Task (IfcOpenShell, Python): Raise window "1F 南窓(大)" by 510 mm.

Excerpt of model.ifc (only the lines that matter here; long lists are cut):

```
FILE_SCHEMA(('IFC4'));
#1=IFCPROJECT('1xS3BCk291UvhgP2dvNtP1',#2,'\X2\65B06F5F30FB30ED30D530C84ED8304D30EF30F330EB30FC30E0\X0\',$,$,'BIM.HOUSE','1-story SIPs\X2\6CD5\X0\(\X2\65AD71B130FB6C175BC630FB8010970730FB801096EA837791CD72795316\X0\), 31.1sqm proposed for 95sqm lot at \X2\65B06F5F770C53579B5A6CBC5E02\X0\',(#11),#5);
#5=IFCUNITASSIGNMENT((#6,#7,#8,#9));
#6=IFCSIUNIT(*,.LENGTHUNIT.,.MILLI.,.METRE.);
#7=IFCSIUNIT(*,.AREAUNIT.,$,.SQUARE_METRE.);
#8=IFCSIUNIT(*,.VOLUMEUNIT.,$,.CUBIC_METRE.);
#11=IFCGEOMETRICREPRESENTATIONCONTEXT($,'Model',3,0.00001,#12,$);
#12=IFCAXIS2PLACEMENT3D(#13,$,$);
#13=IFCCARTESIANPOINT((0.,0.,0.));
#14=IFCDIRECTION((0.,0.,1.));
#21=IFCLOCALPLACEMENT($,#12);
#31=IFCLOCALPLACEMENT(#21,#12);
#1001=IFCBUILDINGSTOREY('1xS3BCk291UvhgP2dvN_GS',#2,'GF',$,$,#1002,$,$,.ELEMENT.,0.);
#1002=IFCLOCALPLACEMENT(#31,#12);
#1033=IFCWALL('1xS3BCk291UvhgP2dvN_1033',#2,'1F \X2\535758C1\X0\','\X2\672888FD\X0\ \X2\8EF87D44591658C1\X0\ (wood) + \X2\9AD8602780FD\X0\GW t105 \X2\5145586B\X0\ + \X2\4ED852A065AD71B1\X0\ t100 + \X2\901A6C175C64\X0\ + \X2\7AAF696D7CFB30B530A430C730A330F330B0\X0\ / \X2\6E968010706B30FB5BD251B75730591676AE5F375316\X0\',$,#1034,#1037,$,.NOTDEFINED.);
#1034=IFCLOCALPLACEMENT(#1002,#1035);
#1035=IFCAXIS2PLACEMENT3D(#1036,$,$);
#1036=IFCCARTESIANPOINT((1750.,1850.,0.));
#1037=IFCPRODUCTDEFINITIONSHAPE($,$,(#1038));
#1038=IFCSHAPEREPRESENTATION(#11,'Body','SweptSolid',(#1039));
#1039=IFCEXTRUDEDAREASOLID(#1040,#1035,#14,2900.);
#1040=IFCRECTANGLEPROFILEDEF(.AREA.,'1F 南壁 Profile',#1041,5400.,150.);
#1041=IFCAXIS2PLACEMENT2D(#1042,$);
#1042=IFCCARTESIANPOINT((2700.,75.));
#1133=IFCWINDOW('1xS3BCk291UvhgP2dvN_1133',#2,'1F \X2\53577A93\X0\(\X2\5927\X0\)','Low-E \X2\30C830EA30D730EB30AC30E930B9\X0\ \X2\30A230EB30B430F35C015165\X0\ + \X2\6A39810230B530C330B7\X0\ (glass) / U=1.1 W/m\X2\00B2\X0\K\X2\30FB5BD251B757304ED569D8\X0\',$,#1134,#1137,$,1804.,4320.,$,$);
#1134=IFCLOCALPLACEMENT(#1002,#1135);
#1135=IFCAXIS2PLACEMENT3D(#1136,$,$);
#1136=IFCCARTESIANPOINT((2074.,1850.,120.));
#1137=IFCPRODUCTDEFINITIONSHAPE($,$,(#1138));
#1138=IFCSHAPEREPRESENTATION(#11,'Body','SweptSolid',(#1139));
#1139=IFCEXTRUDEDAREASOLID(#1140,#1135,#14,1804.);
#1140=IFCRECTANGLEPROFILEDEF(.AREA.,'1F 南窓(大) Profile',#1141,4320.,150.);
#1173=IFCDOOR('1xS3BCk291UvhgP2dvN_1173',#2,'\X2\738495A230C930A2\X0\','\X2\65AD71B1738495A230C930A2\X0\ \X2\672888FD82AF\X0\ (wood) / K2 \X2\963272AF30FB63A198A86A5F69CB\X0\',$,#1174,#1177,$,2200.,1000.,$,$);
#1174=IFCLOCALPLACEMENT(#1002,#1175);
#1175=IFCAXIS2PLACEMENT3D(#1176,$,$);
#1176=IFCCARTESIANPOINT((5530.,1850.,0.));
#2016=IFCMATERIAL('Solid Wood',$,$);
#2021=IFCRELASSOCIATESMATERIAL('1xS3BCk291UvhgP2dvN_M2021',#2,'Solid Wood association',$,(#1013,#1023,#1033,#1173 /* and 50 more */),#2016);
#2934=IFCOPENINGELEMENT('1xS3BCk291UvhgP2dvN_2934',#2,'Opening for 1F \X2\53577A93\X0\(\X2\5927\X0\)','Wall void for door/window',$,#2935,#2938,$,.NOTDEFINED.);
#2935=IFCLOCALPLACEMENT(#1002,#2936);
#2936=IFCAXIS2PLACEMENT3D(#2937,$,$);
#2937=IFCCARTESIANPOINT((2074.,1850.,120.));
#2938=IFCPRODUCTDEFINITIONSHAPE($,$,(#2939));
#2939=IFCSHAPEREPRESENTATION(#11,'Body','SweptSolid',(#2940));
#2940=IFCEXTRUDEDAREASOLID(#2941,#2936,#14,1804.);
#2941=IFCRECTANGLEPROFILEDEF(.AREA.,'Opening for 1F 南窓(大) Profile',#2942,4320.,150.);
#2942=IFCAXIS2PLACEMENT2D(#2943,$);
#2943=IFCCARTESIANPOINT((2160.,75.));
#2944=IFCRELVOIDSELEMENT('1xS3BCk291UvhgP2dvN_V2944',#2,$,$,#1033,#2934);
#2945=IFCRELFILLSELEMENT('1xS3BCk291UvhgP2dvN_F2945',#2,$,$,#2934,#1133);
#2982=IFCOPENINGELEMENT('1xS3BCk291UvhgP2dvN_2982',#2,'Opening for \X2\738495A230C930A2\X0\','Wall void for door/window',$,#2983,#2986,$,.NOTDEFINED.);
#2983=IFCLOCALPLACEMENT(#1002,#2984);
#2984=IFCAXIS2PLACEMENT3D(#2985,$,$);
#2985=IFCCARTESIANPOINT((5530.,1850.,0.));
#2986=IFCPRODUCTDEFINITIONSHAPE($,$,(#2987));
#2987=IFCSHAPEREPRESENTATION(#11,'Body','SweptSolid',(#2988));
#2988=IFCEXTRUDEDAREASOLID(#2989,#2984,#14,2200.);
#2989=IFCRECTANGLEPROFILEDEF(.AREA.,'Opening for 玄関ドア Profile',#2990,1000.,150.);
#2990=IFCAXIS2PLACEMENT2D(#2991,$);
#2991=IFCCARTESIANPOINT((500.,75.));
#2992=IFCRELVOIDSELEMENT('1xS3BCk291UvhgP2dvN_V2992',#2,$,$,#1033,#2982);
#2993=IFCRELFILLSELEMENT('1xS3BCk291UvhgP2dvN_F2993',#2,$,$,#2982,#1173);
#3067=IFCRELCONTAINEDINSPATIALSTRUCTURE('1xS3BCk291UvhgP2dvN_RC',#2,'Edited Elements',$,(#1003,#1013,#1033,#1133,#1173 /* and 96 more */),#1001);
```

```python
import numpy as np
import ifcopenshell
import ifcopenshell.api.geometry
import ifcopenshell.util.placement
import ifcopenshell.util.unit

model = ifcopenshell.open("model.ifc")
unit_scale = ifcopenshell.util.unit.calculate_unit_scale(model)

window = model.by_guid("1xS3BCk291UvhgP2dvN_1133")
opening = window.FillsVoids[0].RelatingOpeningElement
dz = 0.51 / unit_scale

shift = np.array([0.0, 0.0, dz])
# The window is not placed relative to its opening, so move both.
for product in (opening, window):
    matrix = ifcopenshell.util.placement.get_local_placement(product.ObjectPlacement)
    matrix[:3, 3] += shift
    ifcopenshell.api.geometry.edit_object_placement(model, product=product, matrix=matrix, is_si=False)

print(f"moved by {dz * unit_scale:+.3f} m")

model.write("model-out.ifc")
```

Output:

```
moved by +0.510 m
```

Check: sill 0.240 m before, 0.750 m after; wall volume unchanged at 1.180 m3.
